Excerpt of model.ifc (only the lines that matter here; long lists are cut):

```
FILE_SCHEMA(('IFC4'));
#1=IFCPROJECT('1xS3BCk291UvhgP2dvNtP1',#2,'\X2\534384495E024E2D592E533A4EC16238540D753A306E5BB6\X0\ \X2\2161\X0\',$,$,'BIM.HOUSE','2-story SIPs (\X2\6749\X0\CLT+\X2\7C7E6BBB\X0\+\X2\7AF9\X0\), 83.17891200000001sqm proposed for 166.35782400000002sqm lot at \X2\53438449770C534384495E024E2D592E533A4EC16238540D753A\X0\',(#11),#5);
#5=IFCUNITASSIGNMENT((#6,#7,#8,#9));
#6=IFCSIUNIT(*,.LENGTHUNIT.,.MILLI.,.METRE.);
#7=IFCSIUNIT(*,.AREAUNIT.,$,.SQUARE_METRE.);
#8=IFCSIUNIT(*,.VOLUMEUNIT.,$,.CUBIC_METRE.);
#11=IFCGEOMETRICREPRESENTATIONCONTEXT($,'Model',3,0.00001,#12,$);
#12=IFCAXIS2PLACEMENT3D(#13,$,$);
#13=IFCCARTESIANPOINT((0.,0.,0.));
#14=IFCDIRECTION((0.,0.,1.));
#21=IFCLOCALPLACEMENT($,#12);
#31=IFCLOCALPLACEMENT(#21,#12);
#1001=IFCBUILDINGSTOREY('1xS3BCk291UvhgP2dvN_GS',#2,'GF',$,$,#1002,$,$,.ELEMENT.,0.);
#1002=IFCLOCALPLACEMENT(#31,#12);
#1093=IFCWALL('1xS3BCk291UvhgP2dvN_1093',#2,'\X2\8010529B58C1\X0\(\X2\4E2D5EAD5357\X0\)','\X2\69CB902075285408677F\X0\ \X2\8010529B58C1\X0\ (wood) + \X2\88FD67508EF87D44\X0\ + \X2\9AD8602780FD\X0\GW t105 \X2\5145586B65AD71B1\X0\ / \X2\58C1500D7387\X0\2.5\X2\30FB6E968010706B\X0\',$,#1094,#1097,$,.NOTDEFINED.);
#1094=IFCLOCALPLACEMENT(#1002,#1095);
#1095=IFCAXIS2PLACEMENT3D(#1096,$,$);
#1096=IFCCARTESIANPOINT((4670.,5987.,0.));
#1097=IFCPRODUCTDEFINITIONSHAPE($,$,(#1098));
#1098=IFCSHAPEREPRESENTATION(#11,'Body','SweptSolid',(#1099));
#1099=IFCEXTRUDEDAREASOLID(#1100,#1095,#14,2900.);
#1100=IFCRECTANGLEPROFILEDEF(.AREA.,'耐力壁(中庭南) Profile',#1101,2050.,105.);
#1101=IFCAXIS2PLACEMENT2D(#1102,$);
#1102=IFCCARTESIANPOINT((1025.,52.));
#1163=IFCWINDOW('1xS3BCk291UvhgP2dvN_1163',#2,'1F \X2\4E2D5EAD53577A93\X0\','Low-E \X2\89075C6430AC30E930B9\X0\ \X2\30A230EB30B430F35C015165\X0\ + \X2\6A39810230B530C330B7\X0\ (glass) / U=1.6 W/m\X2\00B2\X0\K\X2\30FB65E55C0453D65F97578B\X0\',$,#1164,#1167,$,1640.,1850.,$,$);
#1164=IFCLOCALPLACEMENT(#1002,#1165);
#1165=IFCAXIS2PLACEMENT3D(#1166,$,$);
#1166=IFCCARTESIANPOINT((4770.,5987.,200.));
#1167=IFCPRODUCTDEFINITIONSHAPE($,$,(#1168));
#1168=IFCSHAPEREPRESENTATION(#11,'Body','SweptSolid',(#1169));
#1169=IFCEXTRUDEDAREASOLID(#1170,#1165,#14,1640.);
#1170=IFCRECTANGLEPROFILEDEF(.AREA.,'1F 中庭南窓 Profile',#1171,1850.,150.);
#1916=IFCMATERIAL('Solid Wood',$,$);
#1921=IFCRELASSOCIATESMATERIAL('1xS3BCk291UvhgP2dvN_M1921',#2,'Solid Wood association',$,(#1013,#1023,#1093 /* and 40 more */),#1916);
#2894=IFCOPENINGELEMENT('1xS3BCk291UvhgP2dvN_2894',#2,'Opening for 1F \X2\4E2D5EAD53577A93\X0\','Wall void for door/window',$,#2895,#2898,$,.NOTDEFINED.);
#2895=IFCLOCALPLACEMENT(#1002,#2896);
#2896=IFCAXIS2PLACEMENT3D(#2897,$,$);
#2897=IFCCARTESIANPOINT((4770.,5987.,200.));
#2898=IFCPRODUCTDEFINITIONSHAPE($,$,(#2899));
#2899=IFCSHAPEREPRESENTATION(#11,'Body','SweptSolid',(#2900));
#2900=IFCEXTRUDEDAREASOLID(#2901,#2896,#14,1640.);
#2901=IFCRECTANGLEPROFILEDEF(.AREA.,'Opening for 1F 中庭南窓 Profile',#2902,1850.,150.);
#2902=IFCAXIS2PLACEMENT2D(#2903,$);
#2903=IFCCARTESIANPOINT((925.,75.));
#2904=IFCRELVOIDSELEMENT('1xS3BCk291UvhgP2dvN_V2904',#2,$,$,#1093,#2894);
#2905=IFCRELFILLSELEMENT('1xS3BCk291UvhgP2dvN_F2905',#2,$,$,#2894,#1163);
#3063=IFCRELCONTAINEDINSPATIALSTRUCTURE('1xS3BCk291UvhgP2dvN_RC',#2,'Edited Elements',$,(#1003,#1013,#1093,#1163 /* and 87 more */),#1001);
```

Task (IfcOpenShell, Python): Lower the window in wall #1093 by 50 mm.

```python
import numpy as np
import ifcopenshell
import ifcopenshell.api.geometry
import ifcopenshell.util.placement
import ifcopenshell.util.unit

model = ifcopenshell.open("model.ifc")
unit_scale = ifcopenshell.util.unit.calculate_unit_scale(model)

window = model.by_guid("1xS3BCk291UvhgP2dvN_1163")
opening = window.FillsVoids[0].RelatingOpeningElement
dz = -50.0

shift = np.array([0.0, 0.0, dz])
# The window is not placed relative to its opening, so move both.
for product in (opening, window):
    matrix = ifcopenshell.util.placement.get_local_placement(product.ObjectPlacement)
    matrix[:3, 3] += shift
    ifcopenshell.api.geometry.edit_object_placement(model, product=product, matrix=matrix, is_si=False)

print(f"moved by {dz * unit_scale:+.3f} m")

model.write("model_edited.ifc")
```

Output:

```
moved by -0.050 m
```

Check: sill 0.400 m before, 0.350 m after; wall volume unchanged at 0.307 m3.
